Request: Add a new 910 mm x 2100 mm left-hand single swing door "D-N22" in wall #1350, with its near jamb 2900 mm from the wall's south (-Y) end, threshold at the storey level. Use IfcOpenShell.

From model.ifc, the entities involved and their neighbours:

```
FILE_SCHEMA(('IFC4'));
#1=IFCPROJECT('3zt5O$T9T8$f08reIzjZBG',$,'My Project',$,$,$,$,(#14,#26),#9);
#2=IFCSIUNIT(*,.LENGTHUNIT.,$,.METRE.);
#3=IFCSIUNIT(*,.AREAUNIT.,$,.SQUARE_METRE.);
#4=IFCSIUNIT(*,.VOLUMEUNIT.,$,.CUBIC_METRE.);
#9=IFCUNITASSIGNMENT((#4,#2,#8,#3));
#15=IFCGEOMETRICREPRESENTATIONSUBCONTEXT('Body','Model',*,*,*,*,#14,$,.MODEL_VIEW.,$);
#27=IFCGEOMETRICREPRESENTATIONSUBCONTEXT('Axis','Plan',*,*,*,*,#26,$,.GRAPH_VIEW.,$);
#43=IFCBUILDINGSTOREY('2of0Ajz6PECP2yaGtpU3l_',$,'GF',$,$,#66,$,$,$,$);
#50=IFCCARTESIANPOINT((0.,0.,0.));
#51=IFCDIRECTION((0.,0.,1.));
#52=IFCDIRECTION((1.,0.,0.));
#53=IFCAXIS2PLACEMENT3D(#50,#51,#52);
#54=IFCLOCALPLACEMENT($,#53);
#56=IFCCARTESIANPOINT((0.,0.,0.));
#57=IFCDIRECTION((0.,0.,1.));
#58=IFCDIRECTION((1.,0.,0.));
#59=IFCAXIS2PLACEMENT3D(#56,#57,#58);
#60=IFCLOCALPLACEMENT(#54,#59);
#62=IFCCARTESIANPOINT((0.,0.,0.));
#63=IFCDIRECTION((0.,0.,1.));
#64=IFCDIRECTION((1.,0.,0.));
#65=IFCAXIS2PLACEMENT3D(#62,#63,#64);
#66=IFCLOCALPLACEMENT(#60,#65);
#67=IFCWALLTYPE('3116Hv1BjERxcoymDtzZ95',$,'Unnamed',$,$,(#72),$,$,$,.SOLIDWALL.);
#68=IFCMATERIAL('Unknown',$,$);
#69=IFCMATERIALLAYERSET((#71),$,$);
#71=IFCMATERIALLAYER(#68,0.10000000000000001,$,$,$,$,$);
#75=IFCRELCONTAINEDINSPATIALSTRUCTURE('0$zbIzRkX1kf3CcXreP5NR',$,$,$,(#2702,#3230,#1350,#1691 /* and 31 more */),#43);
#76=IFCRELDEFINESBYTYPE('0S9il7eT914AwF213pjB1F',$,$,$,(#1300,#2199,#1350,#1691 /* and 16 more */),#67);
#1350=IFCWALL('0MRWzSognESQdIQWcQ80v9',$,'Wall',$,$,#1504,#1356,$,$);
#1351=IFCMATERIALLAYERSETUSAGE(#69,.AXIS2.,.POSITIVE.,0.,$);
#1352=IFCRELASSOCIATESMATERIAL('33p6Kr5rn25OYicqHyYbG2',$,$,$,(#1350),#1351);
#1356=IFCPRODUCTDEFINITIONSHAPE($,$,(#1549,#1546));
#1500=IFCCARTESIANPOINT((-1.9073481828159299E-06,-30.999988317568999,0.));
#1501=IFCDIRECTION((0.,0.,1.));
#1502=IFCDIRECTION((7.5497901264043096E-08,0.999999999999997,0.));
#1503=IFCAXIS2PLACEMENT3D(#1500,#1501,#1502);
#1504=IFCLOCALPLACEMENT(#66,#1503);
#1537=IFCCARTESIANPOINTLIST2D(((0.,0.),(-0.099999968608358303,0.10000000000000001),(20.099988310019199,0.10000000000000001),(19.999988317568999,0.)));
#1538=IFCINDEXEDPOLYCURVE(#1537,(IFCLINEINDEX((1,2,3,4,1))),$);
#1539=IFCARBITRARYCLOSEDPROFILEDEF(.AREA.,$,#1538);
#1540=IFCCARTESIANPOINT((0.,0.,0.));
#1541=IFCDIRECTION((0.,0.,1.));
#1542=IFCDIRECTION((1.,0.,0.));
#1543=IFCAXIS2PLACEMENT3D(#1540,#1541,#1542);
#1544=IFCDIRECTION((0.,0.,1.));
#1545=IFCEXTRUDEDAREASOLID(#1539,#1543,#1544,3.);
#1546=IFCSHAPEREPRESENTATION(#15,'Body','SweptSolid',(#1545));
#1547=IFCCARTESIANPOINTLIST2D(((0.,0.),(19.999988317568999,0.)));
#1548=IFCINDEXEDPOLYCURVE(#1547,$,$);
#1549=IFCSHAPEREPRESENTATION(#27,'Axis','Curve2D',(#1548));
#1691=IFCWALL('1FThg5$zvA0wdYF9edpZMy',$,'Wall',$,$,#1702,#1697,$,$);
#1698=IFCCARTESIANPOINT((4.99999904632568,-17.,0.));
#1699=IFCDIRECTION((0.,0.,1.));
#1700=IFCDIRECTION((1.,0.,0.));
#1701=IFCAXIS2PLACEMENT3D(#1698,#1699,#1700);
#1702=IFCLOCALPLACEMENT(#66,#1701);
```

```python
import numpy as np
import ifcopenshell
import ifcopenshell.api.feature
import ifcopenshell.api.geometry
import ifcopenshell.api.root
import ifcopenshell.api.spatial
import ifcopenshell.geom
import ifcopenshell.util.element
import ifcopenshell.util.placement
import ifcopenshell.util.representation
import ifcopenshell.util.shape
import ifcopenshell.util.unit

model = ifcopenshell.open("model.ifc")
unit_scale = ifcopenshell.util.unit.calculate_unit_scale(model)
settings = ifcopenshell.geom.settings()


def volume(element):
    """Net volume in cubic metres, openings subtracted."""
    shape = ifcopenshell.geom.create_shape(settings, element)
    return ifcopenshell.util.shape.get_volume(shape.geometry)


wall = model.by_id(1350)
storey = ifcopenshell.util.element.get_container(wall, ifc_class="IfcBuildingStorey")
context = ifcopenshell.util.representation.get_context(model, "Model", "Body", "MODEL_VIEW")
before = volume(wall)

width, height, from_end, sill = 0.91, 2.1, 2.9, 0.0  # metres

# The wall runs along its own X axis, and the end named is its -X end.
wall_shape = ifcopenshell.geom.create_shape(settings, wall)
x, y, z = ifcopenshell.util.shape.get_vertices(wall_shape.geometry).T
start = x.min() + from_end
face, thickness = float(y.min()), float(y.max() - y.min())
wall_matrix = ifcopenshell.util.placement.get_local_placement(wall.ObjectPlacement)
level = ifcopenshell.util.placement.get_local_placement(storey.ObjectPlacement)[2, 3]


def in_wall(x, y):
    """Placement at x, y metres in the wall's axes, at sill height."""
    matrix = wall_matrix.copy()
    matrix[:, 3] = wall_matrix @ np.array([x / unit_scale, y / unit_scale, 0.0, 1.0])
    matrix[2, 3] = level + sill / unit_scale
    return matrix


# Opening: a box that overshoots both wall faces by 50 mm.
opening = ifcopenshell.api.root.create_entity(model, ifc_class="IfcOpeningElement", predefined_type="OPENING")
box = ifcopenshell.api.geometry.add_wall_representation(
    model, context=context, length=width, height=height, thickness=thickness + 0.1
)
ifcopenshell.api.geometry.assign_representation(model, product=opening, representation=box)
ifcopenshell.api.geometry.edit_object_placement(model, product=opening, matrix=in_wall(start, face - 0.05), is_si=False)
ifcopenshell.api.feature.add_feature(model, feature=opening, element=wall)

door = ifcopenshell.api.root.create_entity(model, ifc_class="IfcDoor", name="D-N22", predefined_type="DOOR")
door.OverallWidth, door.OverallHeight = width / unit_scale, height / unit_scale
door.OperationType = "SINGLE_SWING_LEFT"
body = ifcopenshell.api.geometry.add_door_representation(
    model,
    context=context,
    overall_width=door.OverallWidth,
    overall_height=door.OverallHeight,
    operation_type="SINGLE_SWING_LEFT",
    lining_properties={"LiningDepth": thickness / unit_scale, "ThresholdDepth": thickness / unit_scale},
)
ifcopenshell.api.geometry.assign_representation(model, product=door, representation=body)
ifcopenshell.api.spatial.assign_container(model, products=[door], relating_structure=storey)
ifcopenshell.api.feature.add_filling(model, opening=opening, element=door)

# The lining spans the wall, so the door starts at the wall face.
ifcopenshell.api.geometry.edit_object_placement(model, product=door, matrix=in_wall(start, face), is_si=False)

after = volume(wall)

print(f"wall volume {before:.3f} -> {after:.3f} m3")

model.write("model-out.ifc")
```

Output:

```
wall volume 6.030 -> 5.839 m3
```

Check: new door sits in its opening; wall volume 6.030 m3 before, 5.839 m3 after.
